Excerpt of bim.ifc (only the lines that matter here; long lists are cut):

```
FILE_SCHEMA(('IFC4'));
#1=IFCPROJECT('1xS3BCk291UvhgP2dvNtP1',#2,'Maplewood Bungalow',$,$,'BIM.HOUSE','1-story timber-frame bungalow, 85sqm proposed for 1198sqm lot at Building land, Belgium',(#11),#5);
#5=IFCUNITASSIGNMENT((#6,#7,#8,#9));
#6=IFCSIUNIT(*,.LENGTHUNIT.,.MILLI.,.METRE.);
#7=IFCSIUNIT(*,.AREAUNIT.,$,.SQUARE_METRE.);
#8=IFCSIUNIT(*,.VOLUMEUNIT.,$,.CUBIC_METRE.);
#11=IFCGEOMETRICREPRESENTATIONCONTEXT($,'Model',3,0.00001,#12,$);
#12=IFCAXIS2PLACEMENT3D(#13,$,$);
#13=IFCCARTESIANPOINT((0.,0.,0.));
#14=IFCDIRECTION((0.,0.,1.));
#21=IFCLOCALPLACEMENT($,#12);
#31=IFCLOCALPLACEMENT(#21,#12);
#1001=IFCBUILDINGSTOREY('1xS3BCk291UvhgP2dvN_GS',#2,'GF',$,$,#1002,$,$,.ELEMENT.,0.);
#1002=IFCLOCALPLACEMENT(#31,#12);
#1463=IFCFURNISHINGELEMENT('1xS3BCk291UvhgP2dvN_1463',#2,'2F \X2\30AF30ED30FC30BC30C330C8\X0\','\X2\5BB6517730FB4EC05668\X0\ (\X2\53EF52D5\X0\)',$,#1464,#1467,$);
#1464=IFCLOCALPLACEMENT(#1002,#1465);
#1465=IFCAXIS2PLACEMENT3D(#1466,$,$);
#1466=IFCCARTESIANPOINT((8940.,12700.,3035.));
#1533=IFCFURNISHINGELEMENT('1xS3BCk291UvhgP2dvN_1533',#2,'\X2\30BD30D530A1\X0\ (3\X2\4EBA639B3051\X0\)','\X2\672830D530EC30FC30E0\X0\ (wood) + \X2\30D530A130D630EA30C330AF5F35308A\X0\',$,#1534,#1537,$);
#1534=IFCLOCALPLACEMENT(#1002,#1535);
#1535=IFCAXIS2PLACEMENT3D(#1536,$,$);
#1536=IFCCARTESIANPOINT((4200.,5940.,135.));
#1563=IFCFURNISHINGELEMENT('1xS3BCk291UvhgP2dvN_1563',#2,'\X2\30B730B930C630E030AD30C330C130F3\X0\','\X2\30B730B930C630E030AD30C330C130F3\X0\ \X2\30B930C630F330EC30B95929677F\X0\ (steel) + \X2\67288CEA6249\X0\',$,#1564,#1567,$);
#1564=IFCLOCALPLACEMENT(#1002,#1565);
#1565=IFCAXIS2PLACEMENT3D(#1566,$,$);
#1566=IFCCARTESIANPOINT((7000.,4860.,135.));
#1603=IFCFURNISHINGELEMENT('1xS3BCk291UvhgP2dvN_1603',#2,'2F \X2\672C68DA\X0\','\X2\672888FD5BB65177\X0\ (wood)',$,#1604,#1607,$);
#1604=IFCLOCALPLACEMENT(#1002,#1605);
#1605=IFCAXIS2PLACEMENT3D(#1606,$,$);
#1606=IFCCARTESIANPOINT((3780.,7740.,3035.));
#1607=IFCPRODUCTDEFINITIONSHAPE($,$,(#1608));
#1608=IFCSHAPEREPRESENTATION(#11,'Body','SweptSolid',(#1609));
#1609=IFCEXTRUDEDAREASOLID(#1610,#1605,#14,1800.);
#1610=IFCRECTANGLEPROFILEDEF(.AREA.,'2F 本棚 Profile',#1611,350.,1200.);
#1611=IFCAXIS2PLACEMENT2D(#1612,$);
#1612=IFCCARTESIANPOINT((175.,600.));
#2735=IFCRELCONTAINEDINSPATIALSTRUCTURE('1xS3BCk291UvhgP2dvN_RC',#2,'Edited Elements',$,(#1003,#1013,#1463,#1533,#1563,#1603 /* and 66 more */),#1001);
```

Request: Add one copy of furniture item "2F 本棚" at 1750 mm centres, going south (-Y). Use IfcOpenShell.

```python
import numpy as np
import ifcopenshell
import ifcopenshell.api.geometry
import ifcopenshell.api.root
import ifcopenshell.util.element
import ifcopenshell.util.placement
import ifcopenshell.util.unit

model = ifcopenshell.open("bim.ifc")
unit_scale = ifcopenshell.util.unit.calculate_unit_scale(model)


def reuse_history(source, copy):
    """copy_class also copies each property set's owner history, people and application; keep the originals."""
    for rel in copy.IsDefinedBy:
        if rel.is_a("IfcRelDefinesByProperties") and (history := rel.RelatingPropertyDefinition.OwnerHistory):
            rel.RelatingPropertyDefinition.OwnerHistory = source.OwnerHistory
            ifcopenshell.util.element.remove_deep2(model, history)


source = model.by_guid("1xS3BCk291UvhgP2dvN_1603")
base = ifcopenshell.util.placement.get_local_placement(source.ObjectPlacement)
step = np.array([0.0, -1.0, 0.0]) * 1.75 / unit_scale

for i in range(1, 2):
    copy = ifcopenshell.api.root.copy_class(model, product=source)
    copy.Representation = ifcopenshell.util.element.copy_deep(
        model, source.Representation, exclude=["IfcGeometricRepresentationContext", "IfcRepresentationMap"]
    )
    reuse_history(source, copy)
    matrix = base.copy()
    matrix[:3, 3] += i * step
    print("added at", matrix[:3, 3].round(3) + 0.0)
    ifcopenshell.api.geometry.edit_object_placement(model, product=copy, matrix=matrix, is_si=False)

model.write("bim_updated.ifc")
```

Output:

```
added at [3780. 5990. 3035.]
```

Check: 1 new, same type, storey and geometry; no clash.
